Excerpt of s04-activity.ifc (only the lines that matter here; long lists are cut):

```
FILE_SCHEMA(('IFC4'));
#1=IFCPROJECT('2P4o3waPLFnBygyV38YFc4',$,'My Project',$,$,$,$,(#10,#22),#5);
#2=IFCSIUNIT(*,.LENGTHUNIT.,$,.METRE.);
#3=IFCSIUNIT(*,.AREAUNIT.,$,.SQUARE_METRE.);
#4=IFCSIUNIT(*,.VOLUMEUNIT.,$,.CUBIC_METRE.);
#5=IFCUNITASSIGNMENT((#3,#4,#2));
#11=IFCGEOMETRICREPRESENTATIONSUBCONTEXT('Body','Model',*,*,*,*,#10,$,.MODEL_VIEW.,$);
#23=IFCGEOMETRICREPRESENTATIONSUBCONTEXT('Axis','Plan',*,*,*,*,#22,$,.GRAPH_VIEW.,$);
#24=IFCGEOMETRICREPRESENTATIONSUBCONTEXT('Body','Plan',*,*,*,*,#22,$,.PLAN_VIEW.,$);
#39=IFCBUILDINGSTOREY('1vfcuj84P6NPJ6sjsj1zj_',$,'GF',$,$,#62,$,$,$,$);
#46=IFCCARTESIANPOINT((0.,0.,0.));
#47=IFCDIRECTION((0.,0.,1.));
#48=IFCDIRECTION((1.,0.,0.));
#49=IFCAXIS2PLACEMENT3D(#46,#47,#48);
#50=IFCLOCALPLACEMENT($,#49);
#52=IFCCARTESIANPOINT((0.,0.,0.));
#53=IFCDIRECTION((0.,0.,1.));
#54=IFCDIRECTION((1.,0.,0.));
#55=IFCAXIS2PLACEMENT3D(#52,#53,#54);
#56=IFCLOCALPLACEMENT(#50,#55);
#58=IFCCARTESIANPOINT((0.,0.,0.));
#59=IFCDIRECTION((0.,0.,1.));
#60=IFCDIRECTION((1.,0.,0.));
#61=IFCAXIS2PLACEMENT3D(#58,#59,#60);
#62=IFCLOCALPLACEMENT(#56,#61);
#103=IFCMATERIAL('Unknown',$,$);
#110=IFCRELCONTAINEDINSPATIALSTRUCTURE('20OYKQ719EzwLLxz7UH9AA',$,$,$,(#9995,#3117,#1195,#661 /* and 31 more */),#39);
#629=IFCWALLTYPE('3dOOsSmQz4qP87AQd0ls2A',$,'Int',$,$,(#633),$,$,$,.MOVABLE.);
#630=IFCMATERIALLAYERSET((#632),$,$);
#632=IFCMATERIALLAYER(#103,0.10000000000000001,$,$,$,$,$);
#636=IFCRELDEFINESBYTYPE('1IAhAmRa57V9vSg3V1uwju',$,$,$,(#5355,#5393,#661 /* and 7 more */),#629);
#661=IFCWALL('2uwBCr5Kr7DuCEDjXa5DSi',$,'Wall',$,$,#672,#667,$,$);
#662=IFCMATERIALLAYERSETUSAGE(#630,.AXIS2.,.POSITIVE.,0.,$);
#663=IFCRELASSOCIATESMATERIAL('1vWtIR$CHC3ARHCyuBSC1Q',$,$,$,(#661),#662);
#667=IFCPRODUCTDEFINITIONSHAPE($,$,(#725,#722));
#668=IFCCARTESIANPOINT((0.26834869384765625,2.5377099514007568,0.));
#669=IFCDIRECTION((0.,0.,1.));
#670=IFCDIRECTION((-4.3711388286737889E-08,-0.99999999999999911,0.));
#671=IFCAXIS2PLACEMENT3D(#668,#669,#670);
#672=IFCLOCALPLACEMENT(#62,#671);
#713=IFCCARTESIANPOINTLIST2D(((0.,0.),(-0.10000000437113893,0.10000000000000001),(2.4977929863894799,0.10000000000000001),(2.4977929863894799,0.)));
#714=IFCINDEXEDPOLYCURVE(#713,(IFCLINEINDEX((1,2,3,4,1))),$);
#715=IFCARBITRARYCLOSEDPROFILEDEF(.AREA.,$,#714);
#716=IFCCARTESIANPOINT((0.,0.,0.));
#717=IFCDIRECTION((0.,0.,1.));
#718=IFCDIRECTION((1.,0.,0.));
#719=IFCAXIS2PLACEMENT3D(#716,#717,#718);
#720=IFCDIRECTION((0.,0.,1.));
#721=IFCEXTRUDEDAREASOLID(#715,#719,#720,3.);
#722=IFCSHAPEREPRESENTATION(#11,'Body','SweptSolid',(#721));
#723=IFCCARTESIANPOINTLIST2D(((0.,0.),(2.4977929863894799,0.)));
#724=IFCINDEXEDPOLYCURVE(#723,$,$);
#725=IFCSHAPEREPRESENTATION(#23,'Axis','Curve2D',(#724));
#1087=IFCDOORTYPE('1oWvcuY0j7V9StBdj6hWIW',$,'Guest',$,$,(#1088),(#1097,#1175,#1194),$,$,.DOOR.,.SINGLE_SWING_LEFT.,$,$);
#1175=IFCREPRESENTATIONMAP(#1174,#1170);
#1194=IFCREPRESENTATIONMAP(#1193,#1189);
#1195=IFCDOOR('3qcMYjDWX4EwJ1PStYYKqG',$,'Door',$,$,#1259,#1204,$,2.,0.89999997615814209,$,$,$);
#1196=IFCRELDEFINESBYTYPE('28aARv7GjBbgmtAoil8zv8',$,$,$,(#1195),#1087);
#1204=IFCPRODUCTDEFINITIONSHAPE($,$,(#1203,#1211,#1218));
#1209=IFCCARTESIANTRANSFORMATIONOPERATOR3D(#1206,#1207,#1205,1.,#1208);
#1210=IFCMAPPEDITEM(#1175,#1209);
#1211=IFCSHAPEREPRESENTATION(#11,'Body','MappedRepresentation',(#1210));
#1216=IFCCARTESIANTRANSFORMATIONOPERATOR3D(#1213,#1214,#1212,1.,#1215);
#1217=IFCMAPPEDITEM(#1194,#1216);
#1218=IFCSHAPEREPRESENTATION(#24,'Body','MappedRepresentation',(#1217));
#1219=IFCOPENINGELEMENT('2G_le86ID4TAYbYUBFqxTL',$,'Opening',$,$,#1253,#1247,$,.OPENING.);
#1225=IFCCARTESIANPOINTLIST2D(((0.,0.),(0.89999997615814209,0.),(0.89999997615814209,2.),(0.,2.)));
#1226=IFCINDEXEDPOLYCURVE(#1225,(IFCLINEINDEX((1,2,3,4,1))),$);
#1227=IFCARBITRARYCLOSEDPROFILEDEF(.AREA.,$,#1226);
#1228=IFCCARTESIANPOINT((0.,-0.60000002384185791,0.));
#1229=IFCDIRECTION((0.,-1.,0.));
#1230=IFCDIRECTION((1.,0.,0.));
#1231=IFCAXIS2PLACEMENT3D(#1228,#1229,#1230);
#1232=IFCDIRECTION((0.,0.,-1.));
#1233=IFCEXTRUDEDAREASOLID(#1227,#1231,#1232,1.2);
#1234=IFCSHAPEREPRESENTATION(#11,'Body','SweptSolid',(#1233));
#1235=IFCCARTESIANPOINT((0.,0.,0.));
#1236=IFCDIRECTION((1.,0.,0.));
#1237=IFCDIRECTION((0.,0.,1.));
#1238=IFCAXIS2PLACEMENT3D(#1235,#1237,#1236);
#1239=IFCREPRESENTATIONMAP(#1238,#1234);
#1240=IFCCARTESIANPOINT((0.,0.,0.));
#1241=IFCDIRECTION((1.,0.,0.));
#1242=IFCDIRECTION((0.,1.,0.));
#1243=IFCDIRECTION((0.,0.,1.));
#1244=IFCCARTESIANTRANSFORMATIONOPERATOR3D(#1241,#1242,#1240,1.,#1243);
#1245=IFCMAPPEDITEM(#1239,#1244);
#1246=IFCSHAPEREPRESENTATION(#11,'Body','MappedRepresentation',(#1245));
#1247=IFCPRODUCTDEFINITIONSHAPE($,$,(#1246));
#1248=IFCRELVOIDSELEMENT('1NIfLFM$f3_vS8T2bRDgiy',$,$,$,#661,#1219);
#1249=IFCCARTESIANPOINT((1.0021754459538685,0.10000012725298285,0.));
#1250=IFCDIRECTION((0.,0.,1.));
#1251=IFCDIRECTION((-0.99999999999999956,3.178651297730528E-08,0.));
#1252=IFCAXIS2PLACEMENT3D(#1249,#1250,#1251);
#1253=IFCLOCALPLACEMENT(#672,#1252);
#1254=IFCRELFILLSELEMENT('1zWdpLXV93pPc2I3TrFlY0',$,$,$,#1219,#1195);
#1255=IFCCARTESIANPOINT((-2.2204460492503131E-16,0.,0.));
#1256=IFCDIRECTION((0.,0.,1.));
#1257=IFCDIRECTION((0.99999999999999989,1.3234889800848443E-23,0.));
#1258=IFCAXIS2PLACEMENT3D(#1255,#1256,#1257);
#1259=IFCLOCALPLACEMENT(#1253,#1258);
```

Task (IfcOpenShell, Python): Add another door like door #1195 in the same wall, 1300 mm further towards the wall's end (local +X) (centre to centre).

```python
import ifcopenshell
import ifcopenshell.api.feature
import ifcopenshell.api.geometry
import ifcopenshell.api.root
import ifcopenshell.geom
import ifcopenshell.util.element
import ifcopenshell.util.placement
import ifcopenshell.util.shape
import ifcopenshell.util.unit

model = ifcopenshell.open("s04-activity.ifc")
unit_scale = ifcopenshell.util.unit.calculate_unit_scale(model)
settings = ifcopenshell.geom.settings()


def volume(element):
    """Net volume in cubic metres, openings subtracted."""
    shape = ifcopenshell.geom.create_shape(settings, element)
    return ifcopenshell.util.shape.get_volume(shape.geometry)


door = model.by_id(1195)
opening = door.FillsVoids[0].RelatingOpeningElement
wall = opening.VoidsElements[0].RelatingBuildingElement
before = volume(wall)
shift = ifcopenshell.util.placement.get_local_placement(wall.ObjectPlacement)[:3, 0] * 1.3 / unit_scale

# copy_class copies the void relationship, type, container and properties, but no geometry.
new_opening = ifcopenshell.api.root.copy_class(model, product=opening)
new_opening.Representation = ifcopenshell.util.element.copy_deep(
    model, opening.Representation, exclude=["IfcGeometricRepresentationContext", "IfcRepresentationMap"]
)
new_door = ifcopenshell.api.root.copy_class(model, product=door)
new_door.Representation = ifcopenshell.util.element.copy_deep(
    model, door.Representation, exclude=["IfcGeometricRepresentationContext", "IfcRepresentationMap"]
)
ifcopenshell.api.feature.add_filling(model, opening=new_opening, element=new_door)

for old, new in ((opening, new_opening), (door, new_door)):
    matrix = ifcopenshell.util.placement.get_local_placement(old.ObjectPlacement)
    matrix[:3, 3] += shift
    ifcopenshell.api.geometry.edit_object_placement(model, product=new, matrix=matrix, is_si=False)

after = volume(wall)

print(f"wall volume {before:.3f} -> {after:.3f} m3")

model.write("s04-activity_edited.ifc")
```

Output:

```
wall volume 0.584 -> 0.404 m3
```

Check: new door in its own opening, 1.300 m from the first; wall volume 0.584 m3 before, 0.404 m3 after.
